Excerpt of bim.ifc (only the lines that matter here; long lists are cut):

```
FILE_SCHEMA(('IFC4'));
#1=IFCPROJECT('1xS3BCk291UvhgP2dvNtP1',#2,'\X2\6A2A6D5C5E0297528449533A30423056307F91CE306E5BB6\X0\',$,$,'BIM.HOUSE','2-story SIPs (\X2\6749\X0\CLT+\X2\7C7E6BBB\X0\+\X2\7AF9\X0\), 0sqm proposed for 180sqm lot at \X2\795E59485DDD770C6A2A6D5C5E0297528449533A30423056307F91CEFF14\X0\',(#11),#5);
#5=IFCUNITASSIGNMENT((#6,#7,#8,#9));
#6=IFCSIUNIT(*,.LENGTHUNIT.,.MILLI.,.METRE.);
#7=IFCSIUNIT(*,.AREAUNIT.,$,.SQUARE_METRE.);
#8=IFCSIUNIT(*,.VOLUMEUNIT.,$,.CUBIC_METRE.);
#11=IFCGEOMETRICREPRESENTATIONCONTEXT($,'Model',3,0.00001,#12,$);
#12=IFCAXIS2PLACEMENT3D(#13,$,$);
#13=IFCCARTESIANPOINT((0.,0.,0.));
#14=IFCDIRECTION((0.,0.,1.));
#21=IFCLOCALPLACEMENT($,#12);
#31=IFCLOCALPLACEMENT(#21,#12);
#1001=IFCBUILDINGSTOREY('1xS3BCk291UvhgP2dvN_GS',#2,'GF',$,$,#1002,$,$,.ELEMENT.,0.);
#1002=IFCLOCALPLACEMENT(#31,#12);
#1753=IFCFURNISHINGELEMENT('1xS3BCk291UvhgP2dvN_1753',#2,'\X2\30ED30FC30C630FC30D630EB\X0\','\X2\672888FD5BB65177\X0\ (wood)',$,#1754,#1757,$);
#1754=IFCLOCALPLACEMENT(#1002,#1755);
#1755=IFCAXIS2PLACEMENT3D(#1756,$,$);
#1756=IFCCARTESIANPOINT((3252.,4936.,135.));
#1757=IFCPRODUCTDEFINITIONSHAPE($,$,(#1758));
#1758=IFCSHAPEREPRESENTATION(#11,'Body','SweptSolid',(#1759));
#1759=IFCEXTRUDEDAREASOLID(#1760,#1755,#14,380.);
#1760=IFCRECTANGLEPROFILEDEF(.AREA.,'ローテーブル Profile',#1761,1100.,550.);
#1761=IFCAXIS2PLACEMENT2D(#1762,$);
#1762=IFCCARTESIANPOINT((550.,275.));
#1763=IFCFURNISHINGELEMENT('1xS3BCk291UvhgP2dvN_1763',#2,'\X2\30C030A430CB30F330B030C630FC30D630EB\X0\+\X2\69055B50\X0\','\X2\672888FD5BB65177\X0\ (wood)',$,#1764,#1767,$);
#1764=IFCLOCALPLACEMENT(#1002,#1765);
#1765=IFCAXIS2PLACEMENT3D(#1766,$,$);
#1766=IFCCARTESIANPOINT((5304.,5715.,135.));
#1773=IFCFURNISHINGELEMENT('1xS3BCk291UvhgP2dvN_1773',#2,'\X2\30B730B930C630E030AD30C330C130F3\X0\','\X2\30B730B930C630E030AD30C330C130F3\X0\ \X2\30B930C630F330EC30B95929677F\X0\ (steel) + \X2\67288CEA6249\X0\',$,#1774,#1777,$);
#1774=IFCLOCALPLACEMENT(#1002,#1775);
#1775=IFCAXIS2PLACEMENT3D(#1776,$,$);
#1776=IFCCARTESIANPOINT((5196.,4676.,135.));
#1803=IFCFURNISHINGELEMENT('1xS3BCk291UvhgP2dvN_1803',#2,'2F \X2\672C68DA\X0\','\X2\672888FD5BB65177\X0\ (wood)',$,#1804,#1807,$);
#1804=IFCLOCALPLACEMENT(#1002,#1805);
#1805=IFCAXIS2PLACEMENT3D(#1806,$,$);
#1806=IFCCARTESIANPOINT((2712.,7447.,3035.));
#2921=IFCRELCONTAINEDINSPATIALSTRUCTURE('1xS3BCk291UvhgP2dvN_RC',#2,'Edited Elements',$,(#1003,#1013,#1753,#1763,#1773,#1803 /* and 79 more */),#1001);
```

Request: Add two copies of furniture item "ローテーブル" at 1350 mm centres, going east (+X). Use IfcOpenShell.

```python
import numpy as np
import ifcopenshell
import ifcopenshell.api.geometry
import ifcopenshell.api.root
import ifcopenshell.util.element
import ifcopenshell.util.placement
import ifcopenshell.util.unit

model = ifcopenshell.open("bim.ifc")
unit_scale = ifcopenshell.util.unit.calculate_unit_scale(model)


def reuse_history(source, copy):
    """copy_class also copies each property set's owner history, people and application; keep the originals."""
    for rel in copy.IsDefinedBy:
        if rel.is_a("IfcRelDefinesByProperties") and (history := rel.RelatingPropertyDefinition.OwnerHistory):
            rel.RelatingPropertyDefinition.OwnerHistory = source.OwnerHistory
            ifcopenshell.util.element.remove_deep2(model, history)


source = model.by_guid("1xS3BCk291UvhgP2dvN_1753")
base = ifcopenshell.util.placement.get_local_placement(source.ObjectPlacement)
step = np.array([1.0, 0.0, 0.0]) * 1.35 / unit_scale

for i in range(1, 3):
    copy = ifcopenshell.api.root.copy_class(model, product=source)
    copy.Representation = ifcopenshell.util.element.copy_deep(
        model, source.Representation, exclude=["IfcGeometricRepresentationContext", "IfcRepresentationMap"]
    )
    reuse_history(source, copy)
    matrix = base.copy()
    matrix[:3, 3] += i * step
    print("added at", matrix[:3, 3].round(3) + 0.0)
    ifcopenshell.api.geometry.edit_object_placement(model, product=copy, matrix=matrix, is_si=False)

model.write("bim_updated.ifc")
```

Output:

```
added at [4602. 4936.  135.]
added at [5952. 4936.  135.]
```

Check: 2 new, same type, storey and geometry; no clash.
